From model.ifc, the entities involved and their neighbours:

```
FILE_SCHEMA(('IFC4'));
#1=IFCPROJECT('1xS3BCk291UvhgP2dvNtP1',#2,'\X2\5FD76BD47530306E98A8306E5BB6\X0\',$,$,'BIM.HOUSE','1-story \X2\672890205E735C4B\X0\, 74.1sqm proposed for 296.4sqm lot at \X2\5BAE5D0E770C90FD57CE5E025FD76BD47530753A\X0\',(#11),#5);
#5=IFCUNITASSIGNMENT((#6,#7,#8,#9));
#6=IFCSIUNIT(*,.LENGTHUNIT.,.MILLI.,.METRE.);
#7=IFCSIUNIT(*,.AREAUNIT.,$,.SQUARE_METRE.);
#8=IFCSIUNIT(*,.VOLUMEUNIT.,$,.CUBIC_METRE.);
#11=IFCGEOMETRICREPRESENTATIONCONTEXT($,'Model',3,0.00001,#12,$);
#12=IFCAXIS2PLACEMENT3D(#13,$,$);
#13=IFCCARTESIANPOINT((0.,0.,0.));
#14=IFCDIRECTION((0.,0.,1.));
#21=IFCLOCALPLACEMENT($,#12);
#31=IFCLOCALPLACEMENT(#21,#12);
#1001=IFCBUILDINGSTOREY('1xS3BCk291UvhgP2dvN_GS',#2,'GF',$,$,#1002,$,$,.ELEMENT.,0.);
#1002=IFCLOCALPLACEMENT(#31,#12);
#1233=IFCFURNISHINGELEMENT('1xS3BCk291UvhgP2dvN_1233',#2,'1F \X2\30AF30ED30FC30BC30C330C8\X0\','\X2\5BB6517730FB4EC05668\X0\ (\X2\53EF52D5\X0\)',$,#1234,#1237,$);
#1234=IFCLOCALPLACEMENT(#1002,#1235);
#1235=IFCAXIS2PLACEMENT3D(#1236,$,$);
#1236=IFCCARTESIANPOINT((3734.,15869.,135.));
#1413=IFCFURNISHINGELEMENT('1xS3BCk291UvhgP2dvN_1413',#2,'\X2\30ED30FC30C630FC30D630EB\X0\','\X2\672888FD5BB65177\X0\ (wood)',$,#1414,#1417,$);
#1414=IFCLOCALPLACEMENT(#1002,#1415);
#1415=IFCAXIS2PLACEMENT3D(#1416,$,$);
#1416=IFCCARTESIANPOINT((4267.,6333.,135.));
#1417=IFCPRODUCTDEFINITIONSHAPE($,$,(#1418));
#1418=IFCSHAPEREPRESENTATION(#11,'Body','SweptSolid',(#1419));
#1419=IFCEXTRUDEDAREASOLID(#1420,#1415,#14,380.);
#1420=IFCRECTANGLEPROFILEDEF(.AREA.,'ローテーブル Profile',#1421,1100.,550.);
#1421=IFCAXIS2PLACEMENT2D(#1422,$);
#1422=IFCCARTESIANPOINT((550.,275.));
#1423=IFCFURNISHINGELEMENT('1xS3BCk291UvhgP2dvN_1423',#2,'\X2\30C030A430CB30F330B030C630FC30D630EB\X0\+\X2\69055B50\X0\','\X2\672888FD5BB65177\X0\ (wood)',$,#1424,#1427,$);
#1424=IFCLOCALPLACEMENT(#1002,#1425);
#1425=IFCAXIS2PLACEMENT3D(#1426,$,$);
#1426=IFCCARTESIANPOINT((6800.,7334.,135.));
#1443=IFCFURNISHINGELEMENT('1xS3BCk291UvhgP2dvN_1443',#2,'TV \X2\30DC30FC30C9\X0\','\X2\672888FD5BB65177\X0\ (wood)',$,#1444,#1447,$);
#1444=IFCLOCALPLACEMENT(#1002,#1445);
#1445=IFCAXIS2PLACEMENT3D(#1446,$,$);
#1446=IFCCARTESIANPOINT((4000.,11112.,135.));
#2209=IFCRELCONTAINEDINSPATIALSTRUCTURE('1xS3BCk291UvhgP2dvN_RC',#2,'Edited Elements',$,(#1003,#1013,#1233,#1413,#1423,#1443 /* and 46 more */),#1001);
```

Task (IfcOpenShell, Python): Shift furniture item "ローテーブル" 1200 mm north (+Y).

```python
import ifcopenshell
import ifcopenshell.api.geometry
import ifcopenshell.util.placement
import ifcopenshell.util.unit

model = ifcopenshell.open("model.ifc")
unit_scale = ifcopenshell.util.unit.calculate_unit_scale(model)

item = model.by_guid("1xS3BCk291UvhgP2dvN_1413")
matrix = ifcopenshell.util.placement.get_local_placement(item.ObjectPlacement)
matrix[1, 3] += 1.2 / unit_scale
ifcopenshell.api.geometry.edit_object_placement(model, product=item, matrix=matrix, is_si=False)

print(ifcopenshell.util.placement.get_local_placement(item.ObjectPlacement).round(3) + 0.0)

model.write("model_v2.ifc")
```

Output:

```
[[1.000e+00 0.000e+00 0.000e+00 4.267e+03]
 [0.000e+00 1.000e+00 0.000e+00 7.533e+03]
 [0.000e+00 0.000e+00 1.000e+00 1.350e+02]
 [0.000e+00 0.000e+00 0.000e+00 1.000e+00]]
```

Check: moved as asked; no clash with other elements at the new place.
